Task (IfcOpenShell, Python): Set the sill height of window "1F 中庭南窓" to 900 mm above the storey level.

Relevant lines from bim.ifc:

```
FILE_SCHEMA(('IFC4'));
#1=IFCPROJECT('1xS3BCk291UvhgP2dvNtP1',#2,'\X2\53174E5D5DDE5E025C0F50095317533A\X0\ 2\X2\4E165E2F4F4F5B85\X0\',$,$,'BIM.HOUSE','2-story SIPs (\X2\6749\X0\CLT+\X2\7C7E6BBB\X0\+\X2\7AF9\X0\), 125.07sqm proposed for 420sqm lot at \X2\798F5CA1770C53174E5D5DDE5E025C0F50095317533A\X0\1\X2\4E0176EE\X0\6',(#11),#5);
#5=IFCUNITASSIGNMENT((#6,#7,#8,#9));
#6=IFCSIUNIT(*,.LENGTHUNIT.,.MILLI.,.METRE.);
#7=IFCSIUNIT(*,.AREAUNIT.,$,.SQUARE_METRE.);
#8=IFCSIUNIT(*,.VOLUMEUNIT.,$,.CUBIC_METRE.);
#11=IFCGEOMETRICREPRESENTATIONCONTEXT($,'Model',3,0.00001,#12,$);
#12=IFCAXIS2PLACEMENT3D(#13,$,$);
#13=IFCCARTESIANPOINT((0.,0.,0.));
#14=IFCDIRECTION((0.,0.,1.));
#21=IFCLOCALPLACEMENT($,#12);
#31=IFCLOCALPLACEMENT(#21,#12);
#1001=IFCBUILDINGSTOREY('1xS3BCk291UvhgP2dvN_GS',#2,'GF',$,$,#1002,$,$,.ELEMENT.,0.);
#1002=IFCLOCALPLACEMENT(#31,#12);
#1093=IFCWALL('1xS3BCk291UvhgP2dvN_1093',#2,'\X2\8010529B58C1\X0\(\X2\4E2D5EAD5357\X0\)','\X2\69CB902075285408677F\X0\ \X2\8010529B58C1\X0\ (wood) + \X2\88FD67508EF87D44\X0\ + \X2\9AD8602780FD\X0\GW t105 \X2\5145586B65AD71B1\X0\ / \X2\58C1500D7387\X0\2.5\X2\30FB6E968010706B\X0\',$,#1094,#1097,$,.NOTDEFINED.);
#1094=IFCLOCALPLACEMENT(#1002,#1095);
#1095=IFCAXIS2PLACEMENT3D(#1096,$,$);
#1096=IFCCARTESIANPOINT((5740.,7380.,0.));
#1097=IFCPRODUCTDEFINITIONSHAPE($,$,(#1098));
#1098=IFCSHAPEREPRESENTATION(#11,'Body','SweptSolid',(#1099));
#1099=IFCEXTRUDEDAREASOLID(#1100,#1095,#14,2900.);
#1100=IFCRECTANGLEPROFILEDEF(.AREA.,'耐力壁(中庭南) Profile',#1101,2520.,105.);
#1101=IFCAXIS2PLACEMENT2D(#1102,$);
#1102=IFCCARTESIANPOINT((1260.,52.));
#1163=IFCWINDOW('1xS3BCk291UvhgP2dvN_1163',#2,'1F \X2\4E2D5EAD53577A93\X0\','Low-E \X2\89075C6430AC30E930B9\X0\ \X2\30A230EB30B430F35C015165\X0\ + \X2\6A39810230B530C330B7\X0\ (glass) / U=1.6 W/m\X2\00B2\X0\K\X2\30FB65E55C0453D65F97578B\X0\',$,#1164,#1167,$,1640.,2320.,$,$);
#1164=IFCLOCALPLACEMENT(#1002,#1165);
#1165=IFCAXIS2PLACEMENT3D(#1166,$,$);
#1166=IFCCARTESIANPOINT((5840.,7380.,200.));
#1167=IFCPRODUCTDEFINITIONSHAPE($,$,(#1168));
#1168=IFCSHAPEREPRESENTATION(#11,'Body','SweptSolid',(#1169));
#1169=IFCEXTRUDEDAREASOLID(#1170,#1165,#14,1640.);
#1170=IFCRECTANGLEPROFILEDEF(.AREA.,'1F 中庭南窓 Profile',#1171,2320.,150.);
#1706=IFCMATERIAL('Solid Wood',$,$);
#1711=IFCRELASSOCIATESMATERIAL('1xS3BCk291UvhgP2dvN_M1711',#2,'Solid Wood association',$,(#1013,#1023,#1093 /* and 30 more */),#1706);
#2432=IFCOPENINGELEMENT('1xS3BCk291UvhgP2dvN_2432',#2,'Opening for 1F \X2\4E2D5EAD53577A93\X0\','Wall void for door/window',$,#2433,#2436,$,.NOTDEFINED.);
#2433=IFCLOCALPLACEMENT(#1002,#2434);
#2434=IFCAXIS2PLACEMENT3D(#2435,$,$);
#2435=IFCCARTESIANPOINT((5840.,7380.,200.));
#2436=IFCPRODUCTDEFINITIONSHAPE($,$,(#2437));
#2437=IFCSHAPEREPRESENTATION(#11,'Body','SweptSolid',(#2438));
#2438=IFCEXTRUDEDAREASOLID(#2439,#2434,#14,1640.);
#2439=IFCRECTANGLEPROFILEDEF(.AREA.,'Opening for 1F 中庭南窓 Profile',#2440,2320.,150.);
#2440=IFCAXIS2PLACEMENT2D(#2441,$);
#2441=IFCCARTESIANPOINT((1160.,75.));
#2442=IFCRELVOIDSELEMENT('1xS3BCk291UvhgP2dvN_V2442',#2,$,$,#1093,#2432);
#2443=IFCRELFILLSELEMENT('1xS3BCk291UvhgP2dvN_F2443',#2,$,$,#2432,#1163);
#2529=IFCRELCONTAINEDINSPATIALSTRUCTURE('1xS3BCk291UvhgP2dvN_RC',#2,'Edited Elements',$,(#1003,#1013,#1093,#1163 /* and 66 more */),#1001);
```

```python
import numpy as np
import ifcopenshell
import ifcopenshell.api.geometry
import ifcopenshell.geom
import ifcopenshell.util.element
import ifcopenshell.util.placement
import ifcopenshell.util.shape
import ifcopenshell.util.unit

model = ifcopenshell.open("bim.ifc")
unit_scale = ifcopenshell.util.unit.calculate_unit_scale(model)

window = model.by_guid("1xS3BCk291UvhgP2dvN_1163")
opening = window.FillsVoids[0].RelatingOpeningElement
storey = ifcopenshell.util.element.get_container(window, ifc_class="IfcBuildingStorey")
level = ifcopenshell.util.placement.get_local_placement(storey.ObjectPlacement)[2, 3]

# The opening's origin need not be at the sill, so measure its lowest point.
shape = ifcopenshell.geom.create_shape(ifcopenshell.geom.settings(), opening)
bottom = ifcopenshell.util.shape.get_shape_bottom_elevation(shape, shape.geometry) / unit_scale
dz = level + 0.9 / unit_scale - bottom

shift = np.array([0.0, 0.0, dz])
# The window is not placed relative to its opening, so move both.
for product in (opening, window):
    matrix = ifcopenshell.util.placement.get_local_placement(product.ObjectPlacement)
    matrix[:3, 3] += shift
    ifcopenshell.api.geometry.edit_object_placement(model, product=product, matrix=matrix, is_si=False)

print(f"moved by {dz * unit_scale:+.3f} m")

model.write("bim_v2.ifc")
```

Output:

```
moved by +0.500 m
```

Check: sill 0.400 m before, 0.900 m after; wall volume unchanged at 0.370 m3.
